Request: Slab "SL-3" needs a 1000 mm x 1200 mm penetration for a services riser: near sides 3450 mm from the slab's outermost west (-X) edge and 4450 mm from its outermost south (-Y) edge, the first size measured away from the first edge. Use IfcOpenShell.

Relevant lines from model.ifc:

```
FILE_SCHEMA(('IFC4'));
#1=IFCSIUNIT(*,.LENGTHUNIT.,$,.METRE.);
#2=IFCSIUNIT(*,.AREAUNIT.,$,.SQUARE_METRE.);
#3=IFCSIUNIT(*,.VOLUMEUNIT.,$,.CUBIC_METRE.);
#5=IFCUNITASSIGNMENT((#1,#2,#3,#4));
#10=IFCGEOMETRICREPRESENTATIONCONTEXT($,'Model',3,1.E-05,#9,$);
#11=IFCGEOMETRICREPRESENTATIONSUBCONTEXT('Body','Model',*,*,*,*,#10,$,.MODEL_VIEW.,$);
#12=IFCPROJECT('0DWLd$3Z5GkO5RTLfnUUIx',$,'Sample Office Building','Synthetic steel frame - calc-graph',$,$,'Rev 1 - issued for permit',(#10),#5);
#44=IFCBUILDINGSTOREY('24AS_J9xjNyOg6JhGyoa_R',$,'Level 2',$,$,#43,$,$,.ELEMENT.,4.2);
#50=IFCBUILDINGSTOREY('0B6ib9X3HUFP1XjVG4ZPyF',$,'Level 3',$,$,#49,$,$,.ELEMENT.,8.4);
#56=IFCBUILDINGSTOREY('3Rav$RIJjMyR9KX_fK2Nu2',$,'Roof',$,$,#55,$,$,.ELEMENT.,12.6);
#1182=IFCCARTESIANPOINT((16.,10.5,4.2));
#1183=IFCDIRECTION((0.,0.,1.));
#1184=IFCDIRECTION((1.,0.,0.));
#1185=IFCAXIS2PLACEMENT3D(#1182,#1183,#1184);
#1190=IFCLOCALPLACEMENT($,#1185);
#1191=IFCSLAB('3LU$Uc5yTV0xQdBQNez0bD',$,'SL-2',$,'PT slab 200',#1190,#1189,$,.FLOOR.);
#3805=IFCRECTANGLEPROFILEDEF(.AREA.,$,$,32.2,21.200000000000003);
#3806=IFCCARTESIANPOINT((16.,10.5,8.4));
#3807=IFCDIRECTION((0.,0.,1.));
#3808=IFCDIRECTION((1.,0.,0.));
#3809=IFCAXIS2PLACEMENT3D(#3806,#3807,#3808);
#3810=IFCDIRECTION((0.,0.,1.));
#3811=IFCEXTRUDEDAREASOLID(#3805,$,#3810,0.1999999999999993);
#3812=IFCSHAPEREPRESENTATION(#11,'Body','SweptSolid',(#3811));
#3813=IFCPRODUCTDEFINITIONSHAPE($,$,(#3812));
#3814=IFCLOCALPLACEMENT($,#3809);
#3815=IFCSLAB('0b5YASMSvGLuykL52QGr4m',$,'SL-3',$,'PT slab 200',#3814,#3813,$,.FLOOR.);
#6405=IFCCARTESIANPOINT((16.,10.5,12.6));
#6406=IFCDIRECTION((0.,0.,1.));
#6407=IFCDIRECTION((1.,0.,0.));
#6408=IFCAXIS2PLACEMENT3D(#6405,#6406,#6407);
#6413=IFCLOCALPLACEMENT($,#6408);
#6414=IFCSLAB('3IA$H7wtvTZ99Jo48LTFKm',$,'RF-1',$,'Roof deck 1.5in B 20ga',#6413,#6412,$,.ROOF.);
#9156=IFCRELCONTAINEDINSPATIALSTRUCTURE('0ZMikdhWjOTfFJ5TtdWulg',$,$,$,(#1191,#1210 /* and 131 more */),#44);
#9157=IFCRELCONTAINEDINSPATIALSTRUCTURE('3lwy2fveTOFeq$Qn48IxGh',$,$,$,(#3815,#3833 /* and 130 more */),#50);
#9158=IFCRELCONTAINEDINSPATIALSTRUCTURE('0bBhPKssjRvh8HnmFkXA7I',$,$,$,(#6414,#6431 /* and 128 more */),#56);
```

```python
import numpy as np
import ifcopenshell
import ifcopenshell.api.feature
import ifcopenshell.api.geometry
import ifcopenshell.api.root
import ifcopenshell.geom
import ifcopenshell.util.placement
import ifcopenshell.util.representation
import ifcopenshell.util.shape
import ifcopenshell.util.unit

model = ifcopenshell.open("model.ifc")
unit_scale = ifcopenshell.util.unit.calculate_unit_scale(model)
settings = ifcopenshell.geom.settings()


def volume(element):
    """Net volume in cubic metres, openings subtracted."""
    shape = ifcopenshell.geom.create_shape(settings, element)
    return ifcopenshell.util.shape.get_volume(shape.geometry)


slab = model.by_guid("0b5YASMSvGLuykL52QGr4m")
before = volume(slab)

# Extent in the slab's own axes, in metres. The edges named are its -X and -Y sides.
slab_shape = ifcopenshell.geom.create_shape(settings, slab)
vertices = ifcopenshell.util.shape.get_vertices(slab_shape.geometry)
x_min, y_min, bottom = vertices.min(axis=0)
top = vertices[:, 2].max()

opening = ifcopenshell.api.root.create_entity(model, ifc_class="IfcOpeningElement", name="Services riser opening", predefined_type="OPENING")
context = ifcopenshell.util.representation.get_context(model, "Model", "Body", "MODEL_VIEW")
width, depth = 1, 1.2
outline = [(0.0, 0.0), (width, 0.0), (width, depth), (0.0, depth), (0.0, 0.0)]
# Overshoot both faces by 50 mm so the cut is clean.
shape = ifcopenshell.api.geometry.add_slab_representation(
    model, context=context, depth=top - bottom + 0.1, polyline=outline
)
ifcopenshell.api.geometry.assign_representation(model, product=opening, representation=shape)

matrix = ifcopenshell.util.placement.get_local_placement(slab.ObjectPlacement)
matrix[:, 3] = matrix @ np.append(np.array([x_min + 3.45, y_min + 4.45, bottom - 0.05]) / unit_scale, 1.0)
ifcopenshell.api.geometry.edit_object_placement(model, product=opening, matrix=matrix, is_si=False)
ifcopenshell.api.feature.add_feature(model, feature=opening, element=slab)

after = volume(slab)

print(f"slab volume {before:.3f} -> {after:.3f} m3")

model.write("model_edited.ifc")
```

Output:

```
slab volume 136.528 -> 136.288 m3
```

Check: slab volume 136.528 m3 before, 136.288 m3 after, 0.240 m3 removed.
